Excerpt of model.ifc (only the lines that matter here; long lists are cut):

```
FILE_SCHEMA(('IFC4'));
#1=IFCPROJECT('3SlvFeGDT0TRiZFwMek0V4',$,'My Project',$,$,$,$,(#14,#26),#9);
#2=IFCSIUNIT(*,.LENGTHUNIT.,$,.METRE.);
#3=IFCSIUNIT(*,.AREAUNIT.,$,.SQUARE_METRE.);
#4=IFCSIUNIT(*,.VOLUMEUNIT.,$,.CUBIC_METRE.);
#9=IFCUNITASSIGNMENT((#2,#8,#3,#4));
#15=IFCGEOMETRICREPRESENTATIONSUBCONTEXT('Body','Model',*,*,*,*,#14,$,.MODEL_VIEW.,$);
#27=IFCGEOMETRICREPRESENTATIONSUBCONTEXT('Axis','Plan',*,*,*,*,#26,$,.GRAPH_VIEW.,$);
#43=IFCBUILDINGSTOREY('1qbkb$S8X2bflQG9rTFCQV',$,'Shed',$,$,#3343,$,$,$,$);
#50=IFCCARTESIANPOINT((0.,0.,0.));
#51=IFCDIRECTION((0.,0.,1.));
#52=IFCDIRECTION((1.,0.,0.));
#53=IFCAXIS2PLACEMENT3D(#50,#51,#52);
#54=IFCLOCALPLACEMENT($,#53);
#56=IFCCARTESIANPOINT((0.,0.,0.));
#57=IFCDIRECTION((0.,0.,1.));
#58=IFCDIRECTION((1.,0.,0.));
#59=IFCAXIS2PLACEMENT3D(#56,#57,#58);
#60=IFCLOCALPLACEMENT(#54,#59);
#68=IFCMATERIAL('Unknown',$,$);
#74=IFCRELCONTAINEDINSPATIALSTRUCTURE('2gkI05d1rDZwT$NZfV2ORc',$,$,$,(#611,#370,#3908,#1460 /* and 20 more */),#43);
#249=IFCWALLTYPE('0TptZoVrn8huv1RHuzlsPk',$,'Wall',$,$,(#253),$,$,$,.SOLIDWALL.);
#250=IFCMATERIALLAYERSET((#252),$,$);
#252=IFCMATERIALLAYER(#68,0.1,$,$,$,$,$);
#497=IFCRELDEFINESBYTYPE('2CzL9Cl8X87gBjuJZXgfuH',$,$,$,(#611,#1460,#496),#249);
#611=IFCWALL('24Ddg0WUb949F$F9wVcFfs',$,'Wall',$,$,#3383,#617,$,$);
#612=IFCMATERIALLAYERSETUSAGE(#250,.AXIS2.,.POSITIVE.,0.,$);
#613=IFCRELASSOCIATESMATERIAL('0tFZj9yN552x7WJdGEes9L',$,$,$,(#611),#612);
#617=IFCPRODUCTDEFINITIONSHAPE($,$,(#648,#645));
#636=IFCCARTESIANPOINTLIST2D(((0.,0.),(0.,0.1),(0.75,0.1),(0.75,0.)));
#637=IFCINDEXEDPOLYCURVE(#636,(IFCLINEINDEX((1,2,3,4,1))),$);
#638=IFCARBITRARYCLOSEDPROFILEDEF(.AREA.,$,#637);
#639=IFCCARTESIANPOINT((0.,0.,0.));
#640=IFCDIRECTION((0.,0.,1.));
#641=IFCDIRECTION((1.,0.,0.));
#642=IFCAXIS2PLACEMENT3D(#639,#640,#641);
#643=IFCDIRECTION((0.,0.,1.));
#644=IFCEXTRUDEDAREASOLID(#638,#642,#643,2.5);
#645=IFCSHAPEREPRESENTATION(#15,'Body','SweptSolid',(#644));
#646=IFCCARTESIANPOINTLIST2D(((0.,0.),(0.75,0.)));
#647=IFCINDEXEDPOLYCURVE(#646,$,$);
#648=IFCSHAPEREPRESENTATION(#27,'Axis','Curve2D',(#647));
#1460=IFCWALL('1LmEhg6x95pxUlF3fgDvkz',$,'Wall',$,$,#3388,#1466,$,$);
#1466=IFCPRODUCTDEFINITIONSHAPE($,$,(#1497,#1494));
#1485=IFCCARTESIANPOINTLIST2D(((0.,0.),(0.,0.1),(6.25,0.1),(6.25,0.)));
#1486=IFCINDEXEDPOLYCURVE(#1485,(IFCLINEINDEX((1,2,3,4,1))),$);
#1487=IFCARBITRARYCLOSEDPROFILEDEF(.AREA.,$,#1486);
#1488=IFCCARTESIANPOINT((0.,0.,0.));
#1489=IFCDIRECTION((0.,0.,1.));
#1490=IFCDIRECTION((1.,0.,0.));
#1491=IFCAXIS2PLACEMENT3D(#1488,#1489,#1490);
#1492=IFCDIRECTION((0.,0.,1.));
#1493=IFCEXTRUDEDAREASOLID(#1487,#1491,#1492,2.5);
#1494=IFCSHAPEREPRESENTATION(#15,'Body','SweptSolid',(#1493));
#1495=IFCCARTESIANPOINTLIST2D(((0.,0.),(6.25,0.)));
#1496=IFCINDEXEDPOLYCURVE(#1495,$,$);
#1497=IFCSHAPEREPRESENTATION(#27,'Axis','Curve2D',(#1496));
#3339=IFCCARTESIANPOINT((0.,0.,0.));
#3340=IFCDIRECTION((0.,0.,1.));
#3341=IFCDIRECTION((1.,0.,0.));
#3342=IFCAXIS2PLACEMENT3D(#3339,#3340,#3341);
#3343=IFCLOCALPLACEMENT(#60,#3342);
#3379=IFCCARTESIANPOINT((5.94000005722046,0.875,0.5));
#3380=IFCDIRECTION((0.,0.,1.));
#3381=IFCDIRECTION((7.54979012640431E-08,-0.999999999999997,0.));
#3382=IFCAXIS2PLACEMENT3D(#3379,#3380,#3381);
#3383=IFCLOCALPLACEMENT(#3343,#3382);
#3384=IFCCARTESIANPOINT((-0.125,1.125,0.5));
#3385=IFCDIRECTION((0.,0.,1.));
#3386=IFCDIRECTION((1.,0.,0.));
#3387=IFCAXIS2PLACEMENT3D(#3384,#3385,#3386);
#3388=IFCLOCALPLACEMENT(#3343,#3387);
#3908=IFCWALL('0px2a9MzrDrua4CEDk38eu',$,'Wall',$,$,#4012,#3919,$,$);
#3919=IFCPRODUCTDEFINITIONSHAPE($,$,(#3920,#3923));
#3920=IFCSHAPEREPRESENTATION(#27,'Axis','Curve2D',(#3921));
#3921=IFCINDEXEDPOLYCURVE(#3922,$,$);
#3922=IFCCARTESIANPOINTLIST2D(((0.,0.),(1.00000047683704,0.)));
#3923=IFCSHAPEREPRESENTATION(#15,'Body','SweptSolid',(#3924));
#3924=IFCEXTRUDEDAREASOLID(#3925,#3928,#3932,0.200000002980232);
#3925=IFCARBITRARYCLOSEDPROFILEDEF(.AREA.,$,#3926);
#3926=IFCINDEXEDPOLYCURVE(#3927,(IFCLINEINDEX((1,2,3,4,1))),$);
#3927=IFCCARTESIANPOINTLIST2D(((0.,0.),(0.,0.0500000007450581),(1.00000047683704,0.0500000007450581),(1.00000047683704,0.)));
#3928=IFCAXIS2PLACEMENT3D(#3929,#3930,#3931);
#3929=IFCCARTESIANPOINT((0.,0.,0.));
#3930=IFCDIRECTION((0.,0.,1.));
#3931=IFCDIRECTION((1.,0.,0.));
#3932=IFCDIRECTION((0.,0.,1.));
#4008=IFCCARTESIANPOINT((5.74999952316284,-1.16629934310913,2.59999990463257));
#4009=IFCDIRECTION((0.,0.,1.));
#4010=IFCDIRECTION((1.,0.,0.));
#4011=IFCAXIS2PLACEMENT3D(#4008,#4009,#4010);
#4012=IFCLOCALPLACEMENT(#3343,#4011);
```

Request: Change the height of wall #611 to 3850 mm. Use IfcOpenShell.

```python
import ifcopenshell
import ifcopenshell.geom
import ifcopenshell.util.representation
import ifcopenshell.util.shape

model = ifcopenshell.open("model.ifc")
settings = ifcopenshell.geom.settings()


def volume(element):
    """Net volume in cubic metres, openings subtracted."""
    shape = ifcopenshell.geom.create_shape(settings, element)
    return ifcopenshell.util.shape.get_volume(shape.geometry)


wall = model.by_id(611)
before = volume(wall)

body = ifcopenshell.util.representation.get_representation(wall, "Model", "Body")
solid = body.Items[0]
old_height = solid.Depth
solid.Depth = 3.85
after = volume(wall)

print(f"height {old_height:g} -> {solid.Depth:g}, volume {before:.3f} -> {after:.3f} m3")

model.write("model_updated.ifc")
```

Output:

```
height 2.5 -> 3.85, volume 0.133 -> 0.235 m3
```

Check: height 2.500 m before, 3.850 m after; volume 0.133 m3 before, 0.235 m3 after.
